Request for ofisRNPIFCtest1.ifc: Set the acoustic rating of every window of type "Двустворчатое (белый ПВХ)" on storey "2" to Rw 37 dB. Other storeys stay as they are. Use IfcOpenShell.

First a look at what the model holds.

```python
import ifcopenshell
import ifcopenshell.util.element

model = ifcopenshell.open("ofisRNPIFCtest1.ifc")
print(model.schema)
storey = next(s for s in model.by_type("IfcBuildingStorey") if s.Name == "2")
windows = [e for e in ifcopenshell.util.element.get_decomposition(storey) if e.is_a("IfcWindow")]
seen = {}
for e in windows:
    element_type = ifcopenshell.util.element.get_type(e)
    key = (element_type.Name if element_type != e and element_type else None, ifcopenshell.util.element.get_pset(e, "Pset_WindowCommon", "AcousticRating"))
    seen[key] = seen.get(key, 0) + 1
for (name, value), count in sorted(seen.items(), key=str):
    print(count, "x", name, "|", value)
```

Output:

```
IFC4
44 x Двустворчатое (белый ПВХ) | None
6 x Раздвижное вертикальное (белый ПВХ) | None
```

```python
import ifcopenshell
import ifcopenshell.api.pset
import ifcopenshell.util.element

model = ifcopenshell.open("ofisRNPIFCtest1.ifc")

storey = next(s for s in model.by_type("IfcBuildingStorey") if s.Name == "2")
windows = [e for e in ifcopenshell.util.element.get_decomposition(storey) if e.is_a("IfcWindow")]

count = 0
for e in windows:
    element_type = ifcopenshell.util.element.get_type(e)
    if element_type in (None, e) or element_type.Name != "Двустворчатое (белый ПВХ)":
        continue
    # add_pset returns the element's existing set when there is one.
    pset = ifcopenshell.api.pset.add_pset(model, product=e, name="Pset_WindowCommon")
    ifcopenshell.api.pset.edit_pset(model, pset=pset, properties={"AcousticRating": "Rw 37 dB"})
    count += 1

print(count, "windows updated")

model.write("ofisRNPIFCtest1_updated.ifc")
```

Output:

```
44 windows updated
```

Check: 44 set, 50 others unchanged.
